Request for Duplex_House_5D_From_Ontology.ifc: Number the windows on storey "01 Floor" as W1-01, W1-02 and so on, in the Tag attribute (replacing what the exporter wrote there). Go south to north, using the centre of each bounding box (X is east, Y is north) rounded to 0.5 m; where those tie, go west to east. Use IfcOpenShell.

First a look at what the model holds.

```python
import ifcopenshell
import ifcopenshell.util.element
import ifcopenshell.util.placement

model = ifcopenshell.open("Duplex_House_5D_From_Ontology.ifc")
print(model.schema)
storey = next(s for s in model.by_type("IfcBuildingStorey") if s.Name == "01 Floor")
windows = [e for e in ifcopenshell.util.element.get_decomposition(storey) if e.is_a("IfcWindow")]
for e in sorted(windows, key=lambda e: e.id()):
    origin = ifcopenshell.util.placement.get_local_placement(e.ObjectPlacement)[:3, 3]
    print(e.id(), e.Tag, e.Name, origin.round(2) + 0.0, sep=" | ")
```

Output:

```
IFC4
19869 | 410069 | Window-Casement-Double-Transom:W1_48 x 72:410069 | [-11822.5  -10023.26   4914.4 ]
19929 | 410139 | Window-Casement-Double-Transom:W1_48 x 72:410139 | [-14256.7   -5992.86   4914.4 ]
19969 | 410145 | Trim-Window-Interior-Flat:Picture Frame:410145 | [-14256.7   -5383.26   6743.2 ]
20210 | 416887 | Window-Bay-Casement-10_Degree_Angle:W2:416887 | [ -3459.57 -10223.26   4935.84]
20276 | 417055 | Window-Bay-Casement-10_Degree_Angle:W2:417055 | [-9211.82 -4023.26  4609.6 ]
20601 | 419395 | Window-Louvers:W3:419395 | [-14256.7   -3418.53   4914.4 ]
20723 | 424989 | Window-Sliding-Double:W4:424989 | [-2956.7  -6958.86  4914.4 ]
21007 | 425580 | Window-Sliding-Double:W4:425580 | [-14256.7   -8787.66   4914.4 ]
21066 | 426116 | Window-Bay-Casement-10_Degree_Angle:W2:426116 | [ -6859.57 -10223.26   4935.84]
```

```python
import ifcopenshell
import ifcopenshell.geom
import ifcopenshell.util.element
import ifcopenshell.util.shape

model = ifcopenshell.open("Duplex_House_5D_From_Ontology.ifc")
settings = ifcopenshell.geom.settings()
settings.set("use-world-coords", True)


def centre(element):
    shape = ifcopenshell.geom.create_shape(settings, element)
    return ifcopenshell.util.shape.get_bbox_centroid(shape.geometry)


storey = next(s for s in model.by_type("IfcBuildingStorey") if s.Name == "01 Floor")
windows = [e for e in ifcopenshell.util.element.get_decomposition(storey) if e.is_a("IfcWindow")]

# Insertion points can sit at a corner or the storey origin, so sort by the geometry (in metres).
centres = {e: centre(e) for e in windows}
windows.sort(key=lambda e: (round(centres[e][1] / 0.5), centres[e][0]))

for i, e in enumerate(windows, start=1):
    number = f"W1-{i:02d}"
    e.Tag = number
    print(e.id(), number)

model.write("Duplex_House_5D_From_Ontology_updated.ifc")
```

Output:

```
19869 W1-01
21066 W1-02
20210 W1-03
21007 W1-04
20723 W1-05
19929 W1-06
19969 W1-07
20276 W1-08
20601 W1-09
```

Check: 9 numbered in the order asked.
